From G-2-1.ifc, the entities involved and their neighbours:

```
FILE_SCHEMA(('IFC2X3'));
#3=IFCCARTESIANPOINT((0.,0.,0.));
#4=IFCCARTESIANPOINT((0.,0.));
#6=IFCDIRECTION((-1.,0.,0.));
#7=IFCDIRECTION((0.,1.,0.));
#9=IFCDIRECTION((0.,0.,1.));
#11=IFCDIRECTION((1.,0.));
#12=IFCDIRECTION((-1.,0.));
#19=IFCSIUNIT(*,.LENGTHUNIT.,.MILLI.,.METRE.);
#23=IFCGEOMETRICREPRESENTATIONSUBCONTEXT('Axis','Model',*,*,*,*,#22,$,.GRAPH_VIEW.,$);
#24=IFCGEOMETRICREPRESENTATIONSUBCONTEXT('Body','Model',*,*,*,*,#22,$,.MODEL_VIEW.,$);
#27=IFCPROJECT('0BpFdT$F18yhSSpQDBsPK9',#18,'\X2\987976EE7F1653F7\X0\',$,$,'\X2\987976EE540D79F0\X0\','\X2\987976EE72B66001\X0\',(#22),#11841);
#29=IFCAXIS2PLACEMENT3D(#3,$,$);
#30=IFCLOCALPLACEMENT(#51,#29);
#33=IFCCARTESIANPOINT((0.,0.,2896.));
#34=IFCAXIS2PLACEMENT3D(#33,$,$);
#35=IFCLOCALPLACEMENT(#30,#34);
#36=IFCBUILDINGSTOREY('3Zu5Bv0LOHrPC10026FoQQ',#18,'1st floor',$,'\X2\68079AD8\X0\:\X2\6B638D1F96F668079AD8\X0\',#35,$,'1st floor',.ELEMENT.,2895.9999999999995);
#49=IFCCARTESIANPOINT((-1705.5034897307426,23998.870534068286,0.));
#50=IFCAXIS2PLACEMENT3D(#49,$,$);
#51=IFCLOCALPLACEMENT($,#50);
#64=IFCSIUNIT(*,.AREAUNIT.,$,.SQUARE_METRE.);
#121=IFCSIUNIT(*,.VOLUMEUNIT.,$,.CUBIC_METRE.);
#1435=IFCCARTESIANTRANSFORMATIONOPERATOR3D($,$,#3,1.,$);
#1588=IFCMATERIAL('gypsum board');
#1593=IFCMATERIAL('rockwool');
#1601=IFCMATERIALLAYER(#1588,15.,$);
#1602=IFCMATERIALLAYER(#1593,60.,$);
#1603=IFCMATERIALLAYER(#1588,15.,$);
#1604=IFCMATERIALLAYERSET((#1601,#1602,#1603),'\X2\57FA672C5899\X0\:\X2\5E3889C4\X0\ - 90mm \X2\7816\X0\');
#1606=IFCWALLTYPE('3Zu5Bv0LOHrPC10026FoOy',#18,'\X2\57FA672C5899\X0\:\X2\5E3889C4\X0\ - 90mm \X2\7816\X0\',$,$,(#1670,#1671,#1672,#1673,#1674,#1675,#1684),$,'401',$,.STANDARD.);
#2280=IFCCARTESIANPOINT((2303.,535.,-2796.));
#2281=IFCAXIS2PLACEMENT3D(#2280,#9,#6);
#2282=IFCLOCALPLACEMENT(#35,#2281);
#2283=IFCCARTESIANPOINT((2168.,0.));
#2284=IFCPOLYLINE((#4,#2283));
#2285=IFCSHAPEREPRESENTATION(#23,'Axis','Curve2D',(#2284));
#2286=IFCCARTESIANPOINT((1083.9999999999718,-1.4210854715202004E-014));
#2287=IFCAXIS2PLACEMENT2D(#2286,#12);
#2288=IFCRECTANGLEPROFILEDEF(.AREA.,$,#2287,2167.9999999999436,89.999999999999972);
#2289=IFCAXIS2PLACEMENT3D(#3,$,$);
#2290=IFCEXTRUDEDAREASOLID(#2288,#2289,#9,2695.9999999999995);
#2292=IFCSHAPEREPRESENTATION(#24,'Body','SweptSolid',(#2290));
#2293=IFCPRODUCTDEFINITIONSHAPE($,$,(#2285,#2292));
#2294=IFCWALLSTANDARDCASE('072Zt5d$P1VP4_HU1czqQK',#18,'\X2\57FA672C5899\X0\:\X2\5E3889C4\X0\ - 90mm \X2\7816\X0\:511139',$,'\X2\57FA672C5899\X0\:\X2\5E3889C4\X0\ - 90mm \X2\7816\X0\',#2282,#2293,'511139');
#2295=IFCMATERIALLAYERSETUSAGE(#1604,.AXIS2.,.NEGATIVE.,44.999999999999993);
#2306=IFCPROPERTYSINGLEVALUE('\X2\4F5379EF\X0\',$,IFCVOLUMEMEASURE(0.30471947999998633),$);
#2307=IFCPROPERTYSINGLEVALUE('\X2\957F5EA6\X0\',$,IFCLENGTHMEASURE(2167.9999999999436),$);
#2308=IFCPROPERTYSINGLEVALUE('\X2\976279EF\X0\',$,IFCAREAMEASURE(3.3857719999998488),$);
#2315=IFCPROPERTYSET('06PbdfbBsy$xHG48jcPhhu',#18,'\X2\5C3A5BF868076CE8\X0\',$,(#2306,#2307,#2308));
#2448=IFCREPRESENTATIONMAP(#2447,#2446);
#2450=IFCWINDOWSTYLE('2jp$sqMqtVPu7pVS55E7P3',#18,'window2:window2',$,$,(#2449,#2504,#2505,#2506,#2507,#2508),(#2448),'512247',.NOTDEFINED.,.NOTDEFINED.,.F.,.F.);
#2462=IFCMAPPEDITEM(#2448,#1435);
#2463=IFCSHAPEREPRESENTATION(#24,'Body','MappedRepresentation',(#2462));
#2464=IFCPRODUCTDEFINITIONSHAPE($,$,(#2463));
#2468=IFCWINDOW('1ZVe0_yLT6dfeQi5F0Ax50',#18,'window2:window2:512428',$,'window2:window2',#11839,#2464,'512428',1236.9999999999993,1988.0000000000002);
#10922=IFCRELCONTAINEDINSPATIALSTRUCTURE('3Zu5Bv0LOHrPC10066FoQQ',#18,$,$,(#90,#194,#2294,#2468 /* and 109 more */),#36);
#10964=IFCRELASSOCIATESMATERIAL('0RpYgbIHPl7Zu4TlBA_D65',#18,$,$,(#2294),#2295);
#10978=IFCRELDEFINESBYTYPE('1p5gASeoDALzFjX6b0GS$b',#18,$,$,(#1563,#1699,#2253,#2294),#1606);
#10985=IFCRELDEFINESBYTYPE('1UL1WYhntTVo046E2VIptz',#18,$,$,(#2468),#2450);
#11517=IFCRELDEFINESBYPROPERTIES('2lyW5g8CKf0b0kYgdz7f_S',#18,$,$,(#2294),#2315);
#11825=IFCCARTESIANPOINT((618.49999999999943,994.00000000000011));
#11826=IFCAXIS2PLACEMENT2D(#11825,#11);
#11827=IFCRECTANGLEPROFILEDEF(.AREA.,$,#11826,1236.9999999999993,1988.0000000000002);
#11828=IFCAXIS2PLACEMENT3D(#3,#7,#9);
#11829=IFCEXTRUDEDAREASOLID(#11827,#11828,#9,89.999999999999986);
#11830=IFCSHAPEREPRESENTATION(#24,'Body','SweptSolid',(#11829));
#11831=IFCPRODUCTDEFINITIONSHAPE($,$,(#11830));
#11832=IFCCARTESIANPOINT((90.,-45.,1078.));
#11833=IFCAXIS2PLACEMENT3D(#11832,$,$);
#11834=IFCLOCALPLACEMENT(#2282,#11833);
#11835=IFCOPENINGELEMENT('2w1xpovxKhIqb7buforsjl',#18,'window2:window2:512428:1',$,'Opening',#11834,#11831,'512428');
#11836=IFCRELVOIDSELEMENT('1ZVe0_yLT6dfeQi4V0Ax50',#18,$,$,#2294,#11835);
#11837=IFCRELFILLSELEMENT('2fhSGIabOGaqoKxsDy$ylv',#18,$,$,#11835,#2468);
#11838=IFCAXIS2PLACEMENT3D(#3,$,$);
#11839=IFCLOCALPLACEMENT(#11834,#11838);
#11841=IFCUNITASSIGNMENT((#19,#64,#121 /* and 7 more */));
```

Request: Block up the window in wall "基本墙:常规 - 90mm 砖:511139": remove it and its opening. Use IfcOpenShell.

```python
import ifcopenshell
import ifcopenshell.api.feature
import ifcopenshell.api.pset
import ifcopenshell.api.root
import ifcopenshell.geom
import ifcopenshell.util.element
import ifcopenshell.util.shape
import ifcopenshell.util.unit

model = ifcopenshell.open("G-2-1.ifc")
area_scale = ifcopenshell.util.unit.calculate_unit_scale(model, "AREAUNIT")
volume_scale = ifcopenshell.util.unit.calculate_unit_scale(model, "VOLUMEUNIT")
settings = ifcopenshell.geom.settings()


def volume(element):
    """Net volume in cubic metres, openings subtracted."""
    shape = ifcopenshell.geom.create_shape(settings, element)
    return ifcopenshell.util.shape.get_volume(shape.geometry)


window = model.by_id(2468)
opening = window.FillsVoids[0].RelatingOpeningElement
wall = opening.VoidsElements[0].RelatingBuildingElement
before = volume(wall)

ifcopenshell.api.root.remove_product(model, product=window)
ifcopenshell.api.feature.remove_feature(model, feature=opening)

after = volume(wall)
thickness = 0.09  # wall thickness in metres

# Update the wall's stored quantities.
pset = model.by_id(ifcopenshell.util.element.get_pset(wall, "尺寸标注", should_inherit=False)["id"])
ifcopenshell.api.pset.edit_pset(model, pset=pset, properties={
    "体积": model.create_entity("IfcVolumeMeasure", after / volume_scale),
    "面积": model.create_entity("IfcAreaMeasure", after / thickness / area_scale),
})

print(f"wall volume {before:.3f} -> {after:.3f} m3")

model.write("G-2-1_rev.ifc")
```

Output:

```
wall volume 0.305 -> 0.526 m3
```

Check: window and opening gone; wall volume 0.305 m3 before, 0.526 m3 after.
